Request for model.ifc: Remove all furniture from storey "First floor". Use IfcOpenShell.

First a look at what the model holds.

```python
import ifcopenshell
import ifcopenshell.util.element

model = ifcopenshell.open("model.ifc")
print(model.schema)
storey = next(s for s in model.by_type("IfcBuildingStorey") if s.Name == "First floor")
furniture = [e for e in ifcopenshell.util.element.get_decomposition(storey) if e.is_a("IfcFurnishingElement")]
seen = {}
for e in furniture:
    element_type = ifcopenshell.util.element.get_type(e)
    name = element_type.Name if element_type not in (None, e) else None
    seen[name] = seen.get(name, 0) + 1
for name, count in sorted(seen.items(), key=str):
    print(count, "x", name)
```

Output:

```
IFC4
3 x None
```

```python
import ifcopenshell
import ifcopenshell.api.root
import ifcopenshell.util.element

model = ifcopenshell.open("model.ifc")

storey = next(s for s in model.by_type("IfcBuildingStorey") if s.Name == "First floor")
furniture = [e for e in ifcopenshell.util.element.get_decomposition(storey) if e.is_a("IfcFurnishingElement")]

for e in furniture:
    ifcopenshell.api.root.remove_product(model, product=e)
print(len(furniture), "removed")

model.write("model_edited.ifc")
```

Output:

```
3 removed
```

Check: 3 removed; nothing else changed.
